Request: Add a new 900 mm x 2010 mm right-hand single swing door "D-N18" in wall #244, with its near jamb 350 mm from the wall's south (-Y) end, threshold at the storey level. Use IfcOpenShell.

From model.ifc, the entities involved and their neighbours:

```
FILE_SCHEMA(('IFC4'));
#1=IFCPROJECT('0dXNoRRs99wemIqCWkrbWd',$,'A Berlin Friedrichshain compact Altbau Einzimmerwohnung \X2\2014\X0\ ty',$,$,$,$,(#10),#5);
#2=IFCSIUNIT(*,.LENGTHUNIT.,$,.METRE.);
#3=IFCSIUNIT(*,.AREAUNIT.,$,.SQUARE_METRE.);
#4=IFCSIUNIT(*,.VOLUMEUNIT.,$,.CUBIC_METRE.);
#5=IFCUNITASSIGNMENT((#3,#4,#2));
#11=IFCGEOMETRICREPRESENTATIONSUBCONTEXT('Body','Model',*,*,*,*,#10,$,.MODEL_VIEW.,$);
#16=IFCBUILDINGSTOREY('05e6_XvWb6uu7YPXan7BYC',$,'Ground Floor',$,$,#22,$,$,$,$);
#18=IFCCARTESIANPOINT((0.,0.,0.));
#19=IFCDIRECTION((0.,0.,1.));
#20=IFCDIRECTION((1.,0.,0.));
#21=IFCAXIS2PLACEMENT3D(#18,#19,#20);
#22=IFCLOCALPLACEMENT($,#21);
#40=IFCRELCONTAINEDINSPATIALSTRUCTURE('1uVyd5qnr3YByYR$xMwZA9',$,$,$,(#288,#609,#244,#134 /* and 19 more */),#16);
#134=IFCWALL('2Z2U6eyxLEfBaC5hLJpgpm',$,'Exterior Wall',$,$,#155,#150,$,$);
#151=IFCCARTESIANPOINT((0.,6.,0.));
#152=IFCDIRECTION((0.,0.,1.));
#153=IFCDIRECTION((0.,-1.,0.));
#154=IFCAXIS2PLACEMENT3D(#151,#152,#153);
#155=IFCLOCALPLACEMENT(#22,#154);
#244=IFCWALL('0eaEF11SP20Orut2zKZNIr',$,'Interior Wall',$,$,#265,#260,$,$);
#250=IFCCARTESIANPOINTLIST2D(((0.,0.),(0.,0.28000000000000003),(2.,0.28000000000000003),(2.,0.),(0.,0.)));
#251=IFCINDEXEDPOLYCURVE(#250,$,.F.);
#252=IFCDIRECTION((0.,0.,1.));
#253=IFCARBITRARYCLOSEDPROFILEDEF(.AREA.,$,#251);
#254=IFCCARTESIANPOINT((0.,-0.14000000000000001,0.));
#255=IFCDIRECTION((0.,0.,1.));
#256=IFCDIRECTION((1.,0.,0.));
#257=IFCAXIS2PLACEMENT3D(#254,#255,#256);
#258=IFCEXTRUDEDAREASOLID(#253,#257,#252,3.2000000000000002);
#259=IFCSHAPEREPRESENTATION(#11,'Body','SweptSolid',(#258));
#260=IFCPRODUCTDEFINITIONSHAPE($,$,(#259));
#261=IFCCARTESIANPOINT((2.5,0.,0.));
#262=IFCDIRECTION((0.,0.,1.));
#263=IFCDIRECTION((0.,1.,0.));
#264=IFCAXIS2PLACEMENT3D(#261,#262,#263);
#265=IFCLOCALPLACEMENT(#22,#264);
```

```python
import numpy as np
import ifcopenshell
import ifcopenshell.api.feature
import ifcopenshell.api.geometry
import ifcopenshell.api.root
import ifcopenshell.api.spatial
import ifcopenshell.geom
import ifcopenshell.util.element
import ifcopenshell.util.placement
import ifcopenshell.util.representation
import ifcopenshell.util.shape
import ifcopenshell.util.unit

model = ifcopenshell.open("model.ifc")
unit_scale = ifcopenshell.util.unit.calculate_unit_scale(model)
settings = ifcopenshell.geom.settings()


def volume(element):
    """Net volume in cubic metres, openings subtracted."""
    shape = ifcopenshell.geom.create_shape(settings, element)
    return ifcopenshell.util.shape.get_volume(shape.geometry)


wall = model.by_guid("0eaEF11SP20Orut2zKZNIr")
storey = ifcopenshell.util.element.get_container(wall, ifc_class="IfcBuildingStorey")
context = ifcopenshell.util.representation.get_context(model, "Model", "Body", "MODEL_VIEW")
before = volume(wall)

width, height, from_end, sill = 0.9, 2.01, 0.35, 0.0  # metres

# The wall runs along its own X axis, and the end named is its -X end.
wall_shape = ifcopenshell.geom.create_shape(settings, wall)
x, y, z = ifcopenshell.util.shape.get_vertices(wall_shape.geometry).T
start = x.min() + from_end
face, thickness = float(y.min()), float(y.max() - y.min())
wall_matrix = ifcopenshell.util.placement.get_local_placement(wall.ObjectPlacement)
level = ifcopenshell.util.placement.get_local_placement(storey.ObjectPlacement)[2, 3]


def in_wall(x, y):
    """Placement at x, y metres in the wall's axes, at sill height."""
    matrix = wall_matrix.copy()
    matrix[:, 3] = wall_matrix @ np.array([x / unit_scale, y / unit_scale, 0.0, 1.0])
    matrix[2, 3] = level + sill / unit_scale
    return matrix


# Opening: a box that overshoots both wall faces by 50 mm.
opening = ifcopenshell.api.root.create_entity(model, ifc_class="IfcOpeningElement", predefined_type="OPENING")
box = ifcopenshell.api.geometry.add_wall_representation(
    model, context=context, length=width, height=height, thickness=thickness + 0.1
)
ifcopenshell.api.geometry.assign_representation(model, product=opening, representation=box)
ifcopenshell.api.geometry.edit_object_placement(model, product=opening, matrix=in_wall(start, face - 0.05), is_si=False)
ifcopenshell.api.feature.add_feature(model, feature=opening, element=wall)

door = ifcopenshell.api.root.create_entity(model, ifc_class="IfcDoor", name="D-N18", predefined_type="DOOR")
door.OverallWidth, door.OverallHeight = width / unit_scale, height / unit_scale
door.OperationType = "SINGLE_SWING_RIGHT"
body = ifcopenshell.api.geometry.add_door_representation(
    model,
    context=context,
    overall_width=door.OverallWidth,
    overall_height=door.OverallHeight,
    operation_type="SINGLE_SWING_RIGHT",
    lining_properties={"LiningDepth": thickness / unit_scale, "ThresholdDepth": thickness / unit_scale},
)
ifcopenshell.api.geometry.assign_representation(model, product=door, representation=body)
ifcopenshell.api.spatial.assign_container(model, products=[door], relating_structure=storey)
ifcopenshell.api.feature.add_filling(model, opening=opening, element=door)

# The lining spans the wall, so the door starts at the wall face.
ifcopenshell.api.geometry.edit_object_placement(model, product=door, matrix=in_wall(start, face), is_si=False)

after = volume(wall)

print(f"wall volume {before:.3f} -> {after:.3f} m3")

model.write("model_updated.ifc")
```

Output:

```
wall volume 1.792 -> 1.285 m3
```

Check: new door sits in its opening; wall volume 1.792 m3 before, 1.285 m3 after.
